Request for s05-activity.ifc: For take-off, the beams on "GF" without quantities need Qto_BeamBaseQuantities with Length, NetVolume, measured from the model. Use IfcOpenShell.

First a look at what the model holds.

```python
import ifcopenshell
import ifcopenshell.util.element
import ifcopenshell.util.unit

model = ifcopenshell.open("s05-activity.ifc")
print(model.schema)
for unit_type in ("LENGTHUNIT", "AREAUNIT", "VOLUMEUNIT"):
    print(unit_type, ifcopenshell.util.unit.calculate_unit_scale(model, unit_type))
storey = next(s for s in model.by_type("IfcBuildingStorey") if s.Name == "GF")
beams = [e for e in ifcopenshell.util.element.get_decomposition(storey) if e.is_a("IfcBeam")]
for e in sorted(beams, key=lambda e: e.id()):
    print(e.id(), e.is_a(), e.Name, list(ifcopenshell.util.element.get_psets(e, qtos_only=True)), sep=" | ")
```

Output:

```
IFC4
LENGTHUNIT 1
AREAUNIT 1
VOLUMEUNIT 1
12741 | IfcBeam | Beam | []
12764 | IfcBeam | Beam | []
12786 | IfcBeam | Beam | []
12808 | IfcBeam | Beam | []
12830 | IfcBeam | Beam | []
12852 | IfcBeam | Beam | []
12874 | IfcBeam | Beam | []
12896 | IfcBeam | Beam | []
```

```python
import ifcopenshell
import ifcopenshell.api.pset
import ifcopenshell.geom
import ifcopenshell.util.element
import ifcopenshell.util.shape
import ifcopenshell.util.unit

model = ifcopenshell.open("s05-activity.ifc")
unit_scale = ifcopenshell.util.unit.calculate_unit_scale(model)
volume_scale = ifcopenshell.util.unit.calculate_unit_scale(model, "VOLUMEUNIT")
settings = ifcopenshell.geom.settings()

storey = next(s for s in model.by_type("IfcBuildingStorey") if s.Name == "GF")
beams = [e for e in ifcopenshell.util.element.get_decomposition(storey) if e.is_a("IfcBeam")]

for e in sorted(beams, key=lambda e: e.id()):
    if ifcopenshell.util.element.get_psets(e, qtos_only=True, should_inherit=False):
        continue
    # Geometry comes back in metres, in the element's own axes.
    shape = ifcopenshell.geom.create_shape(settings, e)
    values = {
        "Length": ifcopenshell.util.shape.get_max_xyz(shape.geometry) / unit_scale,
        "NetVolume": ifcopenshell.util.shape.get_volume(shape.geometry) / volume_scale,
    }
    qto = ifcopenshell.api.pset.add_qto(model, product=e, name="Qto_BeamBaseQuantities")
    ifcopenshell.api.pset.edit_qto(model, qto=qto, properties=values)
    print(e.id(), {k: round(v, 3) for k, v in values.items()})

model.write("s05-activity_rev.ifc")
```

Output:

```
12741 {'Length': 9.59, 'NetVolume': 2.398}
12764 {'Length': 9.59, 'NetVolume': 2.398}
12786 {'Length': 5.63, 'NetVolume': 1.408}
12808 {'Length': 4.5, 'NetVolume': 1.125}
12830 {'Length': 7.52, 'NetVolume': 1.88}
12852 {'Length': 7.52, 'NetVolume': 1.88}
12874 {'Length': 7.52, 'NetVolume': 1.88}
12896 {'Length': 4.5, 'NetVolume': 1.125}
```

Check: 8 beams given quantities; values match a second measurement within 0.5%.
